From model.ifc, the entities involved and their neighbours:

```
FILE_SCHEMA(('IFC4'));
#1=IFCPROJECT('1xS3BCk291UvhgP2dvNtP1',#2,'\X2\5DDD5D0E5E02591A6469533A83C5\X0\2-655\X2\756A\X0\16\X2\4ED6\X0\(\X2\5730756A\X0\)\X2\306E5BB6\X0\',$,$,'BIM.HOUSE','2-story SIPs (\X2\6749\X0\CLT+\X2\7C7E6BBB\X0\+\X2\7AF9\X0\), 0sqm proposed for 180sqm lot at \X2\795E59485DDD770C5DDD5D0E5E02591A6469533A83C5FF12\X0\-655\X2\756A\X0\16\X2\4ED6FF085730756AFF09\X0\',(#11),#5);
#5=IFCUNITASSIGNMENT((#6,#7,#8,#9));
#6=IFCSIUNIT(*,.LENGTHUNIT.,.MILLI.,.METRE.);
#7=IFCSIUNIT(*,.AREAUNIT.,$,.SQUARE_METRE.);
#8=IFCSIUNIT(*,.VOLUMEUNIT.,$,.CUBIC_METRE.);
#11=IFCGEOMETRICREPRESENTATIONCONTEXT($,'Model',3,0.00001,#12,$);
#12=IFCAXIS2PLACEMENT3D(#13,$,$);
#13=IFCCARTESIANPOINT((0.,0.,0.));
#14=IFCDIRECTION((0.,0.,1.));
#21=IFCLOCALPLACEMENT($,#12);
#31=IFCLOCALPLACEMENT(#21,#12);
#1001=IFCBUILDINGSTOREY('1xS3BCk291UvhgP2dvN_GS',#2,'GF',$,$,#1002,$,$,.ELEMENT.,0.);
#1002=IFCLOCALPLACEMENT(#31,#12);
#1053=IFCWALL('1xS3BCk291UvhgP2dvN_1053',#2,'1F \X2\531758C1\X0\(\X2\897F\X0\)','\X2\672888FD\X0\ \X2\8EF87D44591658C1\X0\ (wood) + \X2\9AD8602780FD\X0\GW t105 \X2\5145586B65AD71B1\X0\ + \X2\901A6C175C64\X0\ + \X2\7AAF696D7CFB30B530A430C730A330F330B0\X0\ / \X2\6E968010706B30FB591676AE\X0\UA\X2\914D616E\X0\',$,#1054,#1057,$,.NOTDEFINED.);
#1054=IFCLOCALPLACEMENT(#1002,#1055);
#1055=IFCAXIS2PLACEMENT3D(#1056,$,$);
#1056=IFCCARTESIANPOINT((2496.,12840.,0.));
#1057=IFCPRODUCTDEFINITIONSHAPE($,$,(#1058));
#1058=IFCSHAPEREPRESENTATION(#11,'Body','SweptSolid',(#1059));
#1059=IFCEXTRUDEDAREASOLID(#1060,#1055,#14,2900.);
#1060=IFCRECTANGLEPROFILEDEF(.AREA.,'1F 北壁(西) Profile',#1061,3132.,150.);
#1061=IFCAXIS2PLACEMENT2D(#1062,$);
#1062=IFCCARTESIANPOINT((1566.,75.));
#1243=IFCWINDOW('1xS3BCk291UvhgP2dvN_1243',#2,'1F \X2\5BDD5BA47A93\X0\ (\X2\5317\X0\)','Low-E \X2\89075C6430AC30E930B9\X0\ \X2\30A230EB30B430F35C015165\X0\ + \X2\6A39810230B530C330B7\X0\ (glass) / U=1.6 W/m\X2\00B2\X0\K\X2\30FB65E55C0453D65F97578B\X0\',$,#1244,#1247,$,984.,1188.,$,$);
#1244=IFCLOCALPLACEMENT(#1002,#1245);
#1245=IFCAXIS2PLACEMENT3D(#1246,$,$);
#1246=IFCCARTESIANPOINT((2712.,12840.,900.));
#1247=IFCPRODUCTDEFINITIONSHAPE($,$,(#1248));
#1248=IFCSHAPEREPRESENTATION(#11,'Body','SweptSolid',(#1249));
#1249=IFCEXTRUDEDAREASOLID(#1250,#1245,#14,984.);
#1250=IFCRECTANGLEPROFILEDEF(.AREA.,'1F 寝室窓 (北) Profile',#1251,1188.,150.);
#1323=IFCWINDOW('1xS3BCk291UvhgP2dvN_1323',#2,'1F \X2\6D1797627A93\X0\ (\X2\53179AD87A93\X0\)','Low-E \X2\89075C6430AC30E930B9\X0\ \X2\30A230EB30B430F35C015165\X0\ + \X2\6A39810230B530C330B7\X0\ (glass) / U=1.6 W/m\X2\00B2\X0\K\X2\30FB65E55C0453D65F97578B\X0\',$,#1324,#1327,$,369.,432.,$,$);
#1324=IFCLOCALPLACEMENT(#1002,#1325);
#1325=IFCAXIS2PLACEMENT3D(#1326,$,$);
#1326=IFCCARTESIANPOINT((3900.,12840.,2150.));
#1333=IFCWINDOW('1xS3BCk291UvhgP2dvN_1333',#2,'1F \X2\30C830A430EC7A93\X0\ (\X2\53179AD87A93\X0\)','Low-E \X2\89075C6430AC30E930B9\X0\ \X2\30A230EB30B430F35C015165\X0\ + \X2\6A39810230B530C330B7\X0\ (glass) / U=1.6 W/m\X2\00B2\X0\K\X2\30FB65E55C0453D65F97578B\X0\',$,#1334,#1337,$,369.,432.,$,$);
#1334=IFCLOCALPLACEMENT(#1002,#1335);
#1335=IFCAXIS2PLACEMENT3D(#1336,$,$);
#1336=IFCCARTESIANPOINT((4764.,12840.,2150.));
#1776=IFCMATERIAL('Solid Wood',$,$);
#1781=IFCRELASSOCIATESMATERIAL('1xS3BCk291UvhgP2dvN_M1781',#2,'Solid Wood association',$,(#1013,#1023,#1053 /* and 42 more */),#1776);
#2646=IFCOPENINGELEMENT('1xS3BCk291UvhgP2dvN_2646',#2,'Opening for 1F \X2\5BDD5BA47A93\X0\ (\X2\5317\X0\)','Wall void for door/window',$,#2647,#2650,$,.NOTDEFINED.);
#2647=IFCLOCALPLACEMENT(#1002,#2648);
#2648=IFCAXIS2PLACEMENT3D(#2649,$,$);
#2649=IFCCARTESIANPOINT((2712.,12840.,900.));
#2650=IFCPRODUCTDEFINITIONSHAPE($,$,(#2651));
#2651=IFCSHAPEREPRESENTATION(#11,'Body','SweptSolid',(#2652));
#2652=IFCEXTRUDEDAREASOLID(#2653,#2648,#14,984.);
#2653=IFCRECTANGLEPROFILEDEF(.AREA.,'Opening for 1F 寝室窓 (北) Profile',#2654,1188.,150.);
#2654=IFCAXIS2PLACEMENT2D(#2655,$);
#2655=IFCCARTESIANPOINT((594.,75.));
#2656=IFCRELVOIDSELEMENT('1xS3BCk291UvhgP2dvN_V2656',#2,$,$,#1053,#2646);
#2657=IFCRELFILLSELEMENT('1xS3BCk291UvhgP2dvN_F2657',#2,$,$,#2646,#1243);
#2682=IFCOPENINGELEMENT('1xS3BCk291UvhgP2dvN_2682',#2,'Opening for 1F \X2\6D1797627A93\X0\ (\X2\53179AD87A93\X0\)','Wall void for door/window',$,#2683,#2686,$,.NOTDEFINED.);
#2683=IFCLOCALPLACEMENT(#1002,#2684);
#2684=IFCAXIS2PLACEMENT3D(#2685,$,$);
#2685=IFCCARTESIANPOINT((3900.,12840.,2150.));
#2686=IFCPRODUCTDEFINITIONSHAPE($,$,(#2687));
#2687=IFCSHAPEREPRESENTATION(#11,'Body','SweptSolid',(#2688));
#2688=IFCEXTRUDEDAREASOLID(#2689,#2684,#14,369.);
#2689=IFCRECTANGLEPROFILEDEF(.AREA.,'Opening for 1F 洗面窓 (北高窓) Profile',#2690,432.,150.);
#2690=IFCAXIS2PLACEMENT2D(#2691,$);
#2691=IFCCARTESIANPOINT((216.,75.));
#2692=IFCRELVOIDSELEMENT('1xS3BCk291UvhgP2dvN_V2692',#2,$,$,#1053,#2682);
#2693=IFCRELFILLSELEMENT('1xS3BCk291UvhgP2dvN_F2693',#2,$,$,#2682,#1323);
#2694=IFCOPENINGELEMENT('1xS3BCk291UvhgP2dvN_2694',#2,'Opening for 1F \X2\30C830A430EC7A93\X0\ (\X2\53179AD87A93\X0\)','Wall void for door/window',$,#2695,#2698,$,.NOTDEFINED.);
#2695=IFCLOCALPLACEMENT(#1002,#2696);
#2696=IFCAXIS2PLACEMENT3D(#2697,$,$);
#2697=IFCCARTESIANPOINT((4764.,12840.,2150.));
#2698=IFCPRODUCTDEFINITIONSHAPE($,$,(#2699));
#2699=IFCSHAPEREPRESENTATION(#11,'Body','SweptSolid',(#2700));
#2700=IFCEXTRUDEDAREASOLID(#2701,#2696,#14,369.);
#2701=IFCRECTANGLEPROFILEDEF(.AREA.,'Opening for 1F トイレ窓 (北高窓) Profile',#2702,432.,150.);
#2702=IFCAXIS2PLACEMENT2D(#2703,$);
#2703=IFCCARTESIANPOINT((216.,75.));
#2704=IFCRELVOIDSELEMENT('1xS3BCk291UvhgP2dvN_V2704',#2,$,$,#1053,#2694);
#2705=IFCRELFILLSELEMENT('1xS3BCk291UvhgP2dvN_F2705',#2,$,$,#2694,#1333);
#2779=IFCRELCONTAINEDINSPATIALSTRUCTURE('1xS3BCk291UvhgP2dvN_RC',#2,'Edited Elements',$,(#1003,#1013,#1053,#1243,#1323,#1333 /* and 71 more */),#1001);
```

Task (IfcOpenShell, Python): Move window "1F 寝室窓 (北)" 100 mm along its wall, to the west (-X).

```python
import ifcopenshell
import ifcopenshell.api.geometry
import ifcopenshell.util.placement
import ifcopenshell.util.unit

model = ifcopenshell.open("model.ifc")
unit_scale = ifcopenshell.util.unit.calculate_unit_scale(model)

window = model.by_guid("1xS3BCk291UvhgP2dvN_1243")
opening = window.FillsVoids[0].RelatingOpeningElement
wall = opening.VoidsElements[0].RelatingBuildingElement

wall_matrix = ifcopenshell.util.placement.get_local_placement(wall.ObjectPlacement)
shift = wall_matrix[:3, 0] * -0.1 / unit_scale
before = ifcopenshell.util.placement.get_local_placement(window.ObjectPlacement)[:3, 3].copy()

# The window is not placed relative to its opening, so move both.
for product in (opening, window):
    matrix = ifcopenshell.util.placement.get_local_placement(product.ObjectPlacement)
    matrix[:3, 3] += shift
    ifcopenshell.api.geometry.edit_object_placement(model, product=product, matrix=matrix, is_si=False)

after = ifcopenshell.util.placement.get_local_placement(window.ObjectPlacement)[:3, 3]
print("window moved by", (after - before).round(3) + 0.0)

model.write("model_rev.ifc")
```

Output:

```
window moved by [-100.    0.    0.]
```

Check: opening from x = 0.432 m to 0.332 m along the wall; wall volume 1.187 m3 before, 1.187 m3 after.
